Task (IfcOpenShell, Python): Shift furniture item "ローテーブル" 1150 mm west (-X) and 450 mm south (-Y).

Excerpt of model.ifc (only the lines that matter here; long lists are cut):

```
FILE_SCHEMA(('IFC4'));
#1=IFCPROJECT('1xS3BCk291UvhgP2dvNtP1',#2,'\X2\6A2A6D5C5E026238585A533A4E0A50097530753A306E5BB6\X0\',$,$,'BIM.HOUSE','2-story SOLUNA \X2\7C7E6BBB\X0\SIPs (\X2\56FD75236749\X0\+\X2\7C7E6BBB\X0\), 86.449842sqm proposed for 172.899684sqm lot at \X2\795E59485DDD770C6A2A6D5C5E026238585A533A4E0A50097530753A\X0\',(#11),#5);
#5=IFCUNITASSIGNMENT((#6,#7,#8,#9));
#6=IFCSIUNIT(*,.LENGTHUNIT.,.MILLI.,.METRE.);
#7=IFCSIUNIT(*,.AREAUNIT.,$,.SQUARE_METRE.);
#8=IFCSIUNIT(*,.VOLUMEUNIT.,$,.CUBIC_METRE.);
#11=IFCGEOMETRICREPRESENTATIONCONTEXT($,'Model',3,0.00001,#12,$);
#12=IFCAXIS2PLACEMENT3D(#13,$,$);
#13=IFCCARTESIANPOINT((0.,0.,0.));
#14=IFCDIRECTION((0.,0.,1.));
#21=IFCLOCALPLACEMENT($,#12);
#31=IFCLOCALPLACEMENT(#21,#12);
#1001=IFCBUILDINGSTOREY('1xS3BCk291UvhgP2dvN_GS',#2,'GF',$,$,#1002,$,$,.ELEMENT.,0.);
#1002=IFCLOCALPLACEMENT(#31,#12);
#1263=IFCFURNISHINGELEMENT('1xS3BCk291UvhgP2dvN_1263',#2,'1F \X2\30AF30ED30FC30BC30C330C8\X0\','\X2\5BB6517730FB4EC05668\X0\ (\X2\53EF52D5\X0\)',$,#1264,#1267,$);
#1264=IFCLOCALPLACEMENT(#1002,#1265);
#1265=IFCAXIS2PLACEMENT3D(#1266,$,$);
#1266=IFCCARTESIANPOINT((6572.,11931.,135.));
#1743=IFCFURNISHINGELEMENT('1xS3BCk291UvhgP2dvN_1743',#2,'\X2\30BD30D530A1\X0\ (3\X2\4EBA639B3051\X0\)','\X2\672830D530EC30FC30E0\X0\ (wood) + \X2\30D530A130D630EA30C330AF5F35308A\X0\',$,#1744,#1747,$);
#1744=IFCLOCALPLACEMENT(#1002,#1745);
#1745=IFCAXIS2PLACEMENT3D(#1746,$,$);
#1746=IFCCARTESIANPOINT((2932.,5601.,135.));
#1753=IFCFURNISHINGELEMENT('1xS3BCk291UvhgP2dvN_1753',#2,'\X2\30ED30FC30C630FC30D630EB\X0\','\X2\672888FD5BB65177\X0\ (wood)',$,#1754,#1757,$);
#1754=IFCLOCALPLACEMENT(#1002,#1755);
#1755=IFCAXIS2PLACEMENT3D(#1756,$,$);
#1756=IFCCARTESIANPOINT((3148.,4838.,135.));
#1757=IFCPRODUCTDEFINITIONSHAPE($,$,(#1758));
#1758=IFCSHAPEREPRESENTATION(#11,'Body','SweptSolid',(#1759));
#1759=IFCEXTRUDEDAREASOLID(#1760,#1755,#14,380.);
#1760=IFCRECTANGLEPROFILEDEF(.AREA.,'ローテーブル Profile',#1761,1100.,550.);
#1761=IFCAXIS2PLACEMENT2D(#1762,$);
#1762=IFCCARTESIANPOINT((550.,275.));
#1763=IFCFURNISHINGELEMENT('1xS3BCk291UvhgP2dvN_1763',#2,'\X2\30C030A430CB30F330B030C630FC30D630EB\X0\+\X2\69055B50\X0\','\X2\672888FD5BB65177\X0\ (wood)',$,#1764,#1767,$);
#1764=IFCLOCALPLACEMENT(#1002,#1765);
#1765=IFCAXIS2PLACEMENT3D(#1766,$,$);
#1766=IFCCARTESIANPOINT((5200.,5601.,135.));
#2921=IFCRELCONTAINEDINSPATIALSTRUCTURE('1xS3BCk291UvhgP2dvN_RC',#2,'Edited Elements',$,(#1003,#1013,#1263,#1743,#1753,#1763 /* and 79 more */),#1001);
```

```python
import ifcopenshell
import ifcopenshell.api.geometry
import ifcopenshell.util.placement

model = ifcopenshell.open("model.ifc")

item = model.by_guid("1xS3BCk291UvhgP2dvN_1753")
matrix = ifcopenshell.util.placement.get_local_placement(item.ObjectPlacement)
matrix[0, 3] -= 1150.0
matrix[1, 3] -= 450.0
ifcopenshell.api.geometry.edit_object_placement(model, product=item, matrix=matrix, is_si=False)

print(ifcopenshell.util.placement.get_local_placement(item.ObjectPlacement).round(3) + 0.0)

model.write("model_rev.ifc")
```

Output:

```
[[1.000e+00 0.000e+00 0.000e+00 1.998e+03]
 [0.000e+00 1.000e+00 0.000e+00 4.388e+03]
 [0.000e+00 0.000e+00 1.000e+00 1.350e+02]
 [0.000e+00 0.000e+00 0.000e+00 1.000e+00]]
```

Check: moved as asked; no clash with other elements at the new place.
